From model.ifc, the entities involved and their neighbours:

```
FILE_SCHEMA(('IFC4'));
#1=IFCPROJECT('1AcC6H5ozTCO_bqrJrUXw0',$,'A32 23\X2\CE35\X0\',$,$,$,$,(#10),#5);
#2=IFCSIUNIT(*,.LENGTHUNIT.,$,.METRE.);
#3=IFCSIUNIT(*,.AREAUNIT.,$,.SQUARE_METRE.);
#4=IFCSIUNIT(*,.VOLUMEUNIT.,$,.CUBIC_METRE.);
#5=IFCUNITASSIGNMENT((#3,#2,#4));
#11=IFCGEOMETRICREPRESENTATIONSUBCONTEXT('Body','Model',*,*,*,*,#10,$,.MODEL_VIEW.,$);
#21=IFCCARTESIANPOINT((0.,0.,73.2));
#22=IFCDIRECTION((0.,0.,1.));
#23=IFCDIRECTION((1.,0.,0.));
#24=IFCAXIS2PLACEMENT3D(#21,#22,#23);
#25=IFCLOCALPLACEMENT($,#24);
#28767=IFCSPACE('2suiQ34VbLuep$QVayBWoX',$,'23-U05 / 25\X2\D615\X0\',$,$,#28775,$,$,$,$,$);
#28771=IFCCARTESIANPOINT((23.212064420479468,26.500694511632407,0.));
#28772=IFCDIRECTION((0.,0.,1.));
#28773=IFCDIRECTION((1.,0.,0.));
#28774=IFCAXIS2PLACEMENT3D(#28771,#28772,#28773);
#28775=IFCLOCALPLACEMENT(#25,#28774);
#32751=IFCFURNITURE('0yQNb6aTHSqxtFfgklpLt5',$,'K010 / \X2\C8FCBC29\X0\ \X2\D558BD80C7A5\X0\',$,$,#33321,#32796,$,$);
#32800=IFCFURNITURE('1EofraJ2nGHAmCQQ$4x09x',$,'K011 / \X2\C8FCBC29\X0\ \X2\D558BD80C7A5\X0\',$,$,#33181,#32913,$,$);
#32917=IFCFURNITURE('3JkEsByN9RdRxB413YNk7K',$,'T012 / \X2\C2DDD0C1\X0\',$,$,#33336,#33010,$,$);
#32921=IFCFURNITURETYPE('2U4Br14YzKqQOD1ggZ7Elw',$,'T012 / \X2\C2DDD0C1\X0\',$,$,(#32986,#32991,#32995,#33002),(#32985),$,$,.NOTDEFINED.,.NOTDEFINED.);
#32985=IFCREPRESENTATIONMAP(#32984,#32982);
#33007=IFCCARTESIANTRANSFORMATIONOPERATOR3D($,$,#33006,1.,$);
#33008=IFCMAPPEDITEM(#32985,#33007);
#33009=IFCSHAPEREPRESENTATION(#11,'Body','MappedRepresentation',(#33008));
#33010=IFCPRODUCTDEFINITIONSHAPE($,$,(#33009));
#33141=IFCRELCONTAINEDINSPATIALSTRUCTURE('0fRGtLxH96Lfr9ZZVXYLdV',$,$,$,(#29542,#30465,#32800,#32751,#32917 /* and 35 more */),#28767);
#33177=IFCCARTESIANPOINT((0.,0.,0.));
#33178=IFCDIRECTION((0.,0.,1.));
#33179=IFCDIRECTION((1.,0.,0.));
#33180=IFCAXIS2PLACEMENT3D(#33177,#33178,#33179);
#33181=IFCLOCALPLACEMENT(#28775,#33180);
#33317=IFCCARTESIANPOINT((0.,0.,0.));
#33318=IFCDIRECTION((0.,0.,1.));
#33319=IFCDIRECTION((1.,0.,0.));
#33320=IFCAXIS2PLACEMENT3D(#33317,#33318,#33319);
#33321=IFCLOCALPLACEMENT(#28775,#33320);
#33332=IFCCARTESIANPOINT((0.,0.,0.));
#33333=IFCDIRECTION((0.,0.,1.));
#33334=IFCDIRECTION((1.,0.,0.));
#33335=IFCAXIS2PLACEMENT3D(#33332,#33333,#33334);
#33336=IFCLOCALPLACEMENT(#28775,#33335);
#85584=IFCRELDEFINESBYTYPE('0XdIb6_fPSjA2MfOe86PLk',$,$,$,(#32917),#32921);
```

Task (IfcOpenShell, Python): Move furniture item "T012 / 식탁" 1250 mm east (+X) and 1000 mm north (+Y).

```python
import ifcopenshell
import ifcopenshell.api.geometry
import ifcopenshell.util.placement

model = ifcopenshell.open("model.ifc")

item = model.by_id(32917)
matrix = ifcopenshell.util.placement.get_local_placement(item.ObjectPlacement)
matrix[0, 3] += 1.25
matrix[1, 3] += 1.0
ifcopenshell.api.geometry.edit_object_placement(model, product=item, matrix=matrix, is_si=False)

print(ifcopenshell.util.placement.get_local_placement(item.ObjectPlacement).round(3) + 0.0)

model.write("model_v2.ifc")
```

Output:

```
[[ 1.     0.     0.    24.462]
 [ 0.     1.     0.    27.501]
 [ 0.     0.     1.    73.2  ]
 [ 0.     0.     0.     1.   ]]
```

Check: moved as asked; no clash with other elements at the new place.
